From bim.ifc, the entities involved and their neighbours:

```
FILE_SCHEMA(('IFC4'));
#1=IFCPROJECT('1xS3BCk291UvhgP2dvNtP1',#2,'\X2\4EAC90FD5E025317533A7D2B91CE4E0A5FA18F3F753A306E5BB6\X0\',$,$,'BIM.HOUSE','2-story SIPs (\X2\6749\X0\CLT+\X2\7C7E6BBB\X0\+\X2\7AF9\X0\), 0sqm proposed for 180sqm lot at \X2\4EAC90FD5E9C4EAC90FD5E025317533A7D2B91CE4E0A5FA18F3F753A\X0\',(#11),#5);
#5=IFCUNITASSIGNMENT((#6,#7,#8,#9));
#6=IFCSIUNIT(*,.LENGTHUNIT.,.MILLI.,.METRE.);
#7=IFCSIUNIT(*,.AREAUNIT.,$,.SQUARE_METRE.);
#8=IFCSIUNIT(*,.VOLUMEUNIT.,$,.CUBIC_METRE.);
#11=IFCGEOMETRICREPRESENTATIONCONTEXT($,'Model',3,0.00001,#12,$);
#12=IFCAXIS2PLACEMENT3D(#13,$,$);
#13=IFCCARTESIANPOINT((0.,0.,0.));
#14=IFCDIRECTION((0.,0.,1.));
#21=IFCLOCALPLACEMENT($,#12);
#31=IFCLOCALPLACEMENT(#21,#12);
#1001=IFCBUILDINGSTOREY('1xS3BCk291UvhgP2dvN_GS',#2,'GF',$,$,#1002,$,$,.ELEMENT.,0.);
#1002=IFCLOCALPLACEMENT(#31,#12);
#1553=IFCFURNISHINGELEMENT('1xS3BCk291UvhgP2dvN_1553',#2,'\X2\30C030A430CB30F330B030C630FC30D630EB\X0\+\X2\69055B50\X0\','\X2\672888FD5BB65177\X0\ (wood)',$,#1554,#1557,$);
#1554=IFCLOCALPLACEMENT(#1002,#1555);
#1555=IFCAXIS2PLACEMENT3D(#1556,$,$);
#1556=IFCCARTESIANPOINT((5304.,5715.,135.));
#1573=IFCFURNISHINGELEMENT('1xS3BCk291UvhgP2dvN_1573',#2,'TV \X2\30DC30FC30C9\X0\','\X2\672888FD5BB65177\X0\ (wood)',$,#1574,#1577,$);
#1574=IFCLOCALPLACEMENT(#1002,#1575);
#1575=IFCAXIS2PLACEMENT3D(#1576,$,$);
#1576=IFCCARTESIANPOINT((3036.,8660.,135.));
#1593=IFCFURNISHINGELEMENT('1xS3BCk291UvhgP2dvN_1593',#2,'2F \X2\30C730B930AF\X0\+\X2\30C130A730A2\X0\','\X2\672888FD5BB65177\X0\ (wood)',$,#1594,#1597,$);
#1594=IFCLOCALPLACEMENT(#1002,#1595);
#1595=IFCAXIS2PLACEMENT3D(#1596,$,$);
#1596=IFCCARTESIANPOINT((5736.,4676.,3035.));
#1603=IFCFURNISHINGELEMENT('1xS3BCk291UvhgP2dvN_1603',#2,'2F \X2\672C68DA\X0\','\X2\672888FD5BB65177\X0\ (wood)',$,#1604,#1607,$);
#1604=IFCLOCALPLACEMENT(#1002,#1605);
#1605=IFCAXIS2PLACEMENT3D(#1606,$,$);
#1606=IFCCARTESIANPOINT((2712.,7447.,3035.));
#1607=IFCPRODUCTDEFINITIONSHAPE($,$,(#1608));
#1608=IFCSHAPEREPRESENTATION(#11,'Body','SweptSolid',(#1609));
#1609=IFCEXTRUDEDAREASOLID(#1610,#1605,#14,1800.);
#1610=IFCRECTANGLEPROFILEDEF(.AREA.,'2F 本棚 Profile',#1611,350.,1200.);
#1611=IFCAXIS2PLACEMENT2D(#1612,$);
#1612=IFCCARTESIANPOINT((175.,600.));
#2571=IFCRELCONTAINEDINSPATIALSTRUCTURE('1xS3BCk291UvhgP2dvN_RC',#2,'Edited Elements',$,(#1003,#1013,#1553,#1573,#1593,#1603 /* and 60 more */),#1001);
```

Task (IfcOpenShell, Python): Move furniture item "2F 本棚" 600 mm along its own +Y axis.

```python
import ifcopenshell
import ifcopenshell.api.geometry
import ifcopenshell.util.placement

model = ifcopenshell.open("bim.ifc")

item = model.by_id(1603)
matrix = ifcopenshell.util.placement.get_local_placement(item.ObjectPlacement)
matrix[:3, 3] += matrix[:3, 1] * 600.0
ifcopenshell.api.geometry.edit_object_placement(model, product=item, matrix=matrix, is_si=False)

print(ifcopenshell.util.placement.get_local_placement(item.ObjectPlacement).round(3) + 0.0)

model.write("bim_rev.ifc")
```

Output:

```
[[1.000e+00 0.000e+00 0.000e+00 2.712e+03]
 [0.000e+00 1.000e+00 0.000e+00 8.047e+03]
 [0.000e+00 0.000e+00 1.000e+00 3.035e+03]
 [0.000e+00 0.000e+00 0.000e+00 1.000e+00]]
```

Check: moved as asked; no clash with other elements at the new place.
